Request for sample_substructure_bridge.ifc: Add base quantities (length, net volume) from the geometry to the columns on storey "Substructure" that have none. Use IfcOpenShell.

First a look at what the model holds.

```python
import ifcopenshell
import ifcopenshell.util.element
import ifcopenshell.util.unit

model = ifcopenshell.open("sample_substructure_bridge.ifc")
print(model.schema)
for unit_type in ("LENGTHUNIT", "AREAUNIT", "VOLUMEUNIT"):
    print(unit_type, ifcopenshell.util.unit.calculate_unit_scale(model, unit_type))
storey = next(s for s in model.by_type("IfcBuildingStorey") if s.Name == "Substructure")
columns = [e for e in ifcopenshell.util.element.get_decomposition(storey) if e.is_a("IfcColumn")]
for e in sorted(columns, key=lambda e: e.id()):
    print(e.id(), e.is_a(), e.Name, list(ifcopenshell.util.element.get_psets(e, qtos_only=True)), sep=" | ")
```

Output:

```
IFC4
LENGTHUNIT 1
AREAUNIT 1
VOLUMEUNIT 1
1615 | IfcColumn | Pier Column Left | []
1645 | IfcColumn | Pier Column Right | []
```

```python
import ifcopenshell
import ifcopenshell.api.pset
import ifcopenshell.geom
import ifcopenshell.util.element
import ifcopenshell.util.shape
import ifcopenshell.util.unit

model = ifcopenshell.open("sample_substructure_bridge.ifc")
unit_scale = ifcopenshell.util.unit.calculate_unit_scale(model)
volume_scale = ifcopenshell.util.unit.calculate_unit_scale(model, "VOLUMEUNIT")
settings = ifcopenshell.geom.settings()

storey = next(s for s in model.by_type("IfcBuildingStorey") if s.Name == "Substructure")
columns = [e for e in ifcopenshell.util.element.get_decomposition(storey) if e.is_a("IfcColumn")]

for e in sorted(columns, key=lambda e: e.id()):
    if ifcopenshell.util.element.get_psets(e, qtos_only=True, should_inherit=False):
        continue
    # Geometry comes back in metres, in the element's own axes.
    shape = ifcopenshell.geom.create_shape(settings, e)
    values = {
        "Length": ifcopenshell.util.shape.get_z(shape.geometry) / unit_scale,
        "NetVolume": ifcopenshell.util.shape.get_volume(shape.geometry) / volume_scale,
    }
    qto = ifcopenshell.api.pset.add_qto(model, product=e, name="Qto_ColumnBaseQuantities")
    ifcopenshell.api.pset.edit_qto(model, qto=qto, properties=values)
    print(e.id(), {k: round(v, 3) for k, v in values.items()})

model.write("sample_substructure_bridge_v2.ifc")
```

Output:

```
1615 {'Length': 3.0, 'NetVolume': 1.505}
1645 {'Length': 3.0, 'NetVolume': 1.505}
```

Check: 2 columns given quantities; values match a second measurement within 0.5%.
